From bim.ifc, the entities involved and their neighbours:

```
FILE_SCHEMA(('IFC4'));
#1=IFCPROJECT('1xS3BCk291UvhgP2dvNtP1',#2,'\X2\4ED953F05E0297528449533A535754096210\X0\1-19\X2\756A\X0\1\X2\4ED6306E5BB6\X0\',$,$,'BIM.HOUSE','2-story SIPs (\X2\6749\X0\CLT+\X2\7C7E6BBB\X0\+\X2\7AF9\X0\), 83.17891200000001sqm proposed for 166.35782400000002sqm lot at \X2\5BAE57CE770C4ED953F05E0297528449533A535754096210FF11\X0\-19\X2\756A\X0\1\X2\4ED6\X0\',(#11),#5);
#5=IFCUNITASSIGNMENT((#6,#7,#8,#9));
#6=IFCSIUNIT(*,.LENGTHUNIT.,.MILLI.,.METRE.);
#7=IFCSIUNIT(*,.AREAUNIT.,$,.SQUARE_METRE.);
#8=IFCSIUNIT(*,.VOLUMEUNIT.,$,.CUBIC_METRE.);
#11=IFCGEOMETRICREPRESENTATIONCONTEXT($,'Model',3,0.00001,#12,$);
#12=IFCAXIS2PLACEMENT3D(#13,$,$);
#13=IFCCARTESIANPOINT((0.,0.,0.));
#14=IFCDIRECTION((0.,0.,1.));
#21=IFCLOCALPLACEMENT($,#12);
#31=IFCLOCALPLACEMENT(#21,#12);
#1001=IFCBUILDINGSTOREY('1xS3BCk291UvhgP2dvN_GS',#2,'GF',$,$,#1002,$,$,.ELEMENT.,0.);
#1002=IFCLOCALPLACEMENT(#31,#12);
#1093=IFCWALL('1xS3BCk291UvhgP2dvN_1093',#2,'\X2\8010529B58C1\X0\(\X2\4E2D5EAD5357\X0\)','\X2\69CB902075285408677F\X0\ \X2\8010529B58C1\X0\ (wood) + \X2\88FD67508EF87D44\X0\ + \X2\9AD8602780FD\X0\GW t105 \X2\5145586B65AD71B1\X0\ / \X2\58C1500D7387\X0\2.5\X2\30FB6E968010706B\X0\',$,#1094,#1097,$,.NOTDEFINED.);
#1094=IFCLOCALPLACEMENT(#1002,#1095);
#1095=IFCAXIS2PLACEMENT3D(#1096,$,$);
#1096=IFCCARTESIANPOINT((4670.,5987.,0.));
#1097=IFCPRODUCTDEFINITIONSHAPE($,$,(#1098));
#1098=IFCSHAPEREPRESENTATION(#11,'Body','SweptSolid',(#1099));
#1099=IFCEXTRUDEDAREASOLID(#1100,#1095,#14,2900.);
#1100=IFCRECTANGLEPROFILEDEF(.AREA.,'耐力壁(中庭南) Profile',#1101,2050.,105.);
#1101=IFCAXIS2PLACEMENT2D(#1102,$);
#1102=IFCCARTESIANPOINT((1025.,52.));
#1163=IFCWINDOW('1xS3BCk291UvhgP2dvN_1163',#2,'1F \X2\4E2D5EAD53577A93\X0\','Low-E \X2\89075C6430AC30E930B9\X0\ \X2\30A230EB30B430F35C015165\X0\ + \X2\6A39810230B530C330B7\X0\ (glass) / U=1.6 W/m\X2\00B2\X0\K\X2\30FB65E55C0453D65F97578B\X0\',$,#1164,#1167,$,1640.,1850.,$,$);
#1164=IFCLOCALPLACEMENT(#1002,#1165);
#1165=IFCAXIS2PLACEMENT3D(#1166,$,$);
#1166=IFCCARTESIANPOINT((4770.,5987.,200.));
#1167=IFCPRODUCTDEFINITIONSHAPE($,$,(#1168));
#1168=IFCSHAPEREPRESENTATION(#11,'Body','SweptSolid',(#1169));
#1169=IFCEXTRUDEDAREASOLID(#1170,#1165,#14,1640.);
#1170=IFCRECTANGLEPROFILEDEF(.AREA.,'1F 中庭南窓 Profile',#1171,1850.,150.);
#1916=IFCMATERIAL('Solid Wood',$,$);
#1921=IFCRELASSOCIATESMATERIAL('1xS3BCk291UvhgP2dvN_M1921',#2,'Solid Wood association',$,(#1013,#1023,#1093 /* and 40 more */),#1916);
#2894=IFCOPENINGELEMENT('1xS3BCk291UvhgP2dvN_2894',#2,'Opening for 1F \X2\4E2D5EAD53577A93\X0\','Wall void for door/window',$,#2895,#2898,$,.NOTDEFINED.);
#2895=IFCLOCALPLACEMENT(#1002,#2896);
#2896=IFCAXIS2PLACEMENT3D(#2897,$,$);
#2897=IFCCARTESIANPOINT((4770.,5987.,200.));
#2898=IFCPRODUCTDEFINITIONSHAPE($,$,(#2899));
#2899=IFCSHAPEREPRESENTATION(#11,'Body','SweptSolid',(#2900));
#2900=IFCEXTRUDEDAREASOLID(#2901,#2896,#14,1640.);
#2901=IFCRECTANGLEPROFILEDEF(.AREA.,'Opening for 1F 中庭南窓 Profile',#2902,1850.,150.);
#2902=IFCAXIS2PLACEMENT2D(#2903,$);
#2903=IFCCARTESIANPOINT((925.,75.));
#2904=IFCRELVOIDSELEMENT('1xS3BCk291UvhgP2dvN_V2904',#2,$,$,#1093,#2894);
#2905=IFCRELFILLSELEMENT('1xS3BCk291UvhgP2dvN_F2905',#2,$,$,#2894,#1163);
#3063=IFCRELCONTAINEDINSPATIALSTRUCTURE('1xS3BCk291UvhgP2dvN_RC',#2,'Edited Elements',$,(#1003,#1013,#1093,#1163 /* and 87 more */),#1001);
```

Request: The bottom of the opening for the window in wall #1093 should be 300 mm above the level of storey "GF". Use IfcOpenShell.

```python
import numpy as np
import ifcopenshell
import ifcopenshell.api.geometry
import ifcopenshell.geom
import ifcopenshell.util.element
import ifcopenshell.util.placement
import ifcopenshell.util.shape
import ifcopenshell.util.unit

model = ifcopenshell.open("bim.ifc")
unit_scale = ifcopenshell.util.unit.calculate_unit_scale(model)

window = model.by_id(1163)
opening = window.FillsVoids[0].RelatingOpeningElement
storey = ifcopenshell.util.element.get_container(window, ifc_class="IfcBuildingStorey")
level = ifcopenshell.util.placement.get_local_placement(storey.ObjectPlacement)[2, 3]

# The opening's origin need not be at the sill, so measure its lowest point.
shape = ifcopenshell.geom.create_shape(ifcopenshell.geom.settings(), opening)
bottom = ifcopenshell.util.shape.get_shape_bottom_elevation(shape, shape.geometry) / unit_scale
dz = level + 300.0 - bottom

shift = np.array([0.0, 0.0, dz])
# The window is not placed relative to its opening, so move both.
for product in (opening, window):
    matrix = ifcopenshell.util.placement.get_local_placement(product.ObjectPlacement)
    matrix[:3, 3] += shift
    ifcopenshell.api.geometry.edit_object_placement(model, product=product, matrix=matrix, is_si=False)

print(f"moved by {dz * unit_scale:+.3f} m")

model.write("bim_rev.ifc")
```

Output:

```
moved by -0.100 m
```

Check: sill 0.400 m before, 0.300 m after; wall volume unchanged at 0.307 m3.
